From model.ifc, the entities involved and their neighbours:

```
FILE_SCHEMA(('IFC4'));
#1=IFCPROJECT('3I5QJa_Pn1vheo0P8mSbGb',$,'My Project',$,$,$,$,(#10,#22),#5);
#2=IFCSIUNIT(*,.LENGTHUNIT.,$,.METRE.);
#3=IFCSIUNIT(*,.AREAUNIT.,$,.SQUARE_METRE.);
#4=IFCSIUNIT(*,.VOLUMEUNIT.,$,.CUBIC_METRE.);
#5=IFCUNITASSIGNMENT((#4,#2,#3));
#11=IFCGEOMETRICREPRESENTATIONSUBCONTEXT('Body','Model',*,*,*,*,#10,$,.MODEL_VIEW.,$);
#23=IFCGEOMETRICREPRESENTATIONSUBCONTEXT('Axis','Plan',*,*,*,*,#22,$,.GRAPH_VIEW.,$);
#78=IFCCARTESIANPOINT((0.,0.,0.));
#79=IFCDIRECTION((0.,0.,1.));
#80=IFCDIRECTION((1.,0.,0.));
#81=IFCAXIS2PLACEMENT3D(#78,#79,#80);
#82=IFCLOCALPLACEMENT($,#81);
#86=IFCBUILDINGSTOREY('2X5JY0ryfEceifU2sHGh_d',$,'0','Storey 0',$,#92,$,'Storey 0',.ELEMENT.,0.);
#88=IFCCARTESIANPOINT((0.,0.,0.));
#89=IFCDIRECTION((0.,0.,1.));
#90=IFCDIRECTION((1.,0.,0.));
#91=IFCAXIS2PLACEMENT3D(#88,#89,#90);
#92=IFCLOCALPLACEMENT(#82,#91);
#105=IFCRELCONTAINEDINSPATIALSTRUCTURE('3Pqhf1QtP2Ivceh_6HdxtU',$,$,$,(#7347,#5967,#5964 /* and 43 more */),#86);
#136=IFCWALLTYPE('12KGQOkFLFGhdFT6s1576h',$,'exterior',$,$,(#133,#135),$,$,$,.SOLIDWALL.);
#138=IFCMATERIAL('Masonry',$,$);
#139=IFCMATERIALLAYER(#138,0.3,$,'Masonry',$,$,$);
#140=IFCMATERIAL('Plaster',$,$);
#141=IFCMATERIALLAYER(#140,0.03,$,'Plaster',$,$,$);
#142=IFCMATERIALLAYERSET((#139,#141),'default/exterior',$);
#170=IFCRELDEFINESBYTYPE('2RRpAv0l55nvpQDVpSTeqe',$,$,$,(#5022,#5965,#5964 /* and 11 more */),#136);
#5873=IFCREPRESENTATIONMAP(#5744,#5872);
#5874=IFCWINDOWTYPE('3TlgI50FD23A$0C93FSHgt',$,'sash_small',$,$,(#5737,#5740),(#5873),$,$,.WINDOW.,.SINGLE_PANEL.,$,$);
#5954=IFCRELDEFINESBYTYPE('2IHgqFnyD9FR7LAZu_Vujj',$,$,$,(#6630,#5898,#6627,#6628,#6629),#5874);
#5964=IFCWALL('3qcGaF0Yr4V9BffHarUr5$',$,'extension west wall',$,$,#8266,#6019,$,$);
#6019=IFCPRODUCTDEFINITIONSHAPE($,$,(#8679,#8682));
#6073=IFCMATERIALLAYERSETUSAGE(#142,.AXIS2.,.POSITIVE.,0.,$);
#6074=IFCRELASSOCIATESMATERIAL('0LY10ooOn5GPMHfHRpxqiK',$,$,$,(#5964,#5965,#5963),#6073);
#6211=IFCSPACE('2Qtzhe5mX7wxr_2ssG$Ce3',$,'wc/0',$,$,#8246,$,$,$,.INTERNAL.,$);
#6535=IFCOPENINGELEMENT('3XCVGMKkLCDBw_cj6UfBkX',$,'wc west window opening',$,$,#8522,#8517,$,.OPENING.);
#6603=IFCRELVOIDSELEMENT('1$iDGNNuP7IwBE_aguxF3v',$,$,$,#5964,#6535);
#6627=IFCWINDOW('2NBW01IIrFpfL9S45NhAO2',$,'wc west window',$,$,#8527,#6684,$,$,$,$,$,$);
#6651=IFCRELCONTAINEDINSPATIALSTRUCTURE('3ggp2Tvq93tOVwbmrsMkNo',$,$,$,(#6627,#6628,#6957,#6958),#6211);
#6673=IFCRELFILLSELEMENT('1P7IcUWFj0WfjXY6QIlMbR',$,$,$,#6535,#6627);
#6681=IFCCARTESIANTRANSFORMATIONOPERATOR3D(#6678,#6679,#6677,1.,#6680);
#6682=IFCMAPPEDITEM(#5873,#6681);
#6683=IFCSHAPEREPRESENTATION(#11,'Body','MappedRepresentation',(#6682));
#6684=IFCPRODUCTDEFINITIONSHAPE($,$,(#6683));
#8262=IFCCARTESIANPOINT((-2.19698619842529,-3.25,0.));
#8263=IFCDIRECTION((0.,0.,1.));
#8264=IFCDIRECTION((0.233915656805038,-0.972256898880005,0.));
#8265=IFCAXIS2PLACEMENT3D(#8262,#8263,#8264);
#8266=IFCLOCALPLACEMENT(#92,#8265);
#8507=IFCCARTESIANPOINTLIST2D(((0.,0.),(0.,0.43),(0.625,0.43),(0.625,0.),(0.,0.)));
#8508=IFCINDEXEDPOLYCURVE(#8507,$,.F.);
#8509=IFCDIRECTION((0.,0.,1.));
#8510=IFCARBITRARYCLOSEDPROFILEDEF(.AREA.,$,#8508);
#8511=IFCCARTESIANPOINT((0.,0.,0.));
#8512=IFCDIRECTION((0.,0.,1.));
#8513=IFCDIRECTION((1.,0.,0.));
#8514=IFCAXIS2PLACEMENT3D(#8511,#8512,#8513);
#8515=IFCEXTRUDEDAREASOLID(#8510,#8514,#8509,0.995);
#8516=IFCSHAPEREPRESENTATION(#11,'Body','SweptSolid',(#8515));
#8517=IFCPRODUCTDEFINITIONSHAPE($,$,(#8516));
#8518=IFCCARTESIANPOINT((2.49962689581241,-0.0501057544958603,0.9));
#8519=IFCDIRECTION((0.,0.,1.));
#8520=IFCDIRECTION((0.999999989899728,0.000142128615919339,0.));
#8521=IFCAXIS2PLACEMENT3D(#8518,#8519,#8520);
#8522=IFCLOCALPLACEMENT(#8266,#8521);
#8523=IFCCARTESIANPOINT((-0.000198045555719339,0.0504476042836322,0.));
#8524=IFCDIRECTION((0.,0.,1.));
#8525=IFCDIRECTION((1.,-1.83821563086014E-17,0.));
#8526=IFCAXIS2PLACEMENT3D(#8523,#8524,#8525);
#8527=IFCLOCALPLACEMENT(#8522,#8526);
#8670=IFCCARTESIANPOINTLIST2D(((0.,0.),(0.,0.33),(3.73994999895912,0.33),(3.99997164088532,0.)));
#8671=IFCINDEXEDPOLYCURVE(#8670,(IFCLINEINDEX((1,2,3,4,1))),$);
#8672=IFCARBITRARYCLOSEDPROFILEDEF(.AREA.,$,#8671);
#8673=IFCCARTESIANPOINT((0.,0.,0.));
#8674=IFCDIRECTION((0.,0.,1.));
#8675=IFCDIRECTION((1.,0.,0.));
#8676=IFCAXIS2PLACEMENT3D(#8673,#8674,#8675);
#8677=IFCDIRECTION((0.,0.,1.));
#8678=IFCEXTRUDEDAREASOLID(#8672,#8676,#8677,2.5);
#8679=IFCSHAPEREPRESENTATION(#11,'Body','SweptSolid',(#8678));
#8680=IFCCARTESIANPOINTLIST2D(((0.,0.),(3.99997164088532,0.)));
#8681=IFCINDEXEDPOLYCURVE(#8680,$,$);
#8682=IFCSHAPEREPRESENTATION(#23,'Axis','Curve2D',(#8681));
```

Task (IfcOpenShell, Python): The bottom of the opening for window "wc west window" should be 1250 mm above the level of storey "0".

```python
import numpy as np
import ifcopenshell
import ifcopenshell.api.geometry
import ifcopenshell.geom
import ifcopenshell.util.element
import ifcopenshell.util.placement
import ifcopenshell.util.shape
import ifcopenshell.util.unit

model = ifcopenshell.open("model.ifc")
unit_scale = ifcopenshell.util.unit.calculate_unit_scale(model)

window = model.by_id(6627)
opening = window.FillsVoids[0].RelatingOpeningElement
storey = ifcopenshell.util.element.get_container(window, ifc_class="IfcBuildingStorey")
level = ifcopenshell.util.placement.get_local_placement(storey.ObjectPlacement)[2, 3]

# The opening's origin need not be at the sill, so measure its lowest point.
shape = ifcopenshell.geom.create_shape(ifcopenshell.geom.settings(), opening)
bottom = ifcopenshell.util.shape.get_shape_bottom_elevation(shape, shape.geometry) / unit_scale
dz = level + 1.25 / unit_scale - bottom

shift = np.array([0.0, 0.0, dz])
# The window is placed relative to its opening, so it follows when the opening moves.
matrix = ifcopenshell.util.placement.get_local_placement(opening.ObjectPlacement)
matrix[:3, 3] += shift
ifcopenshell.api.geometry.edit_object_placement(
    model, product=opening, matrix=matrix, is_si=False, should_transform_children=True
)

print(f"moved by {dz * unit_scale:+.3f} m")

model.write("model_v2.ifc")
```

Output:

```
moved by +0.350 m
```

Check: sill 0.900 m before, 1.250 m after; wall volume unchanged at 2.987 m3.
